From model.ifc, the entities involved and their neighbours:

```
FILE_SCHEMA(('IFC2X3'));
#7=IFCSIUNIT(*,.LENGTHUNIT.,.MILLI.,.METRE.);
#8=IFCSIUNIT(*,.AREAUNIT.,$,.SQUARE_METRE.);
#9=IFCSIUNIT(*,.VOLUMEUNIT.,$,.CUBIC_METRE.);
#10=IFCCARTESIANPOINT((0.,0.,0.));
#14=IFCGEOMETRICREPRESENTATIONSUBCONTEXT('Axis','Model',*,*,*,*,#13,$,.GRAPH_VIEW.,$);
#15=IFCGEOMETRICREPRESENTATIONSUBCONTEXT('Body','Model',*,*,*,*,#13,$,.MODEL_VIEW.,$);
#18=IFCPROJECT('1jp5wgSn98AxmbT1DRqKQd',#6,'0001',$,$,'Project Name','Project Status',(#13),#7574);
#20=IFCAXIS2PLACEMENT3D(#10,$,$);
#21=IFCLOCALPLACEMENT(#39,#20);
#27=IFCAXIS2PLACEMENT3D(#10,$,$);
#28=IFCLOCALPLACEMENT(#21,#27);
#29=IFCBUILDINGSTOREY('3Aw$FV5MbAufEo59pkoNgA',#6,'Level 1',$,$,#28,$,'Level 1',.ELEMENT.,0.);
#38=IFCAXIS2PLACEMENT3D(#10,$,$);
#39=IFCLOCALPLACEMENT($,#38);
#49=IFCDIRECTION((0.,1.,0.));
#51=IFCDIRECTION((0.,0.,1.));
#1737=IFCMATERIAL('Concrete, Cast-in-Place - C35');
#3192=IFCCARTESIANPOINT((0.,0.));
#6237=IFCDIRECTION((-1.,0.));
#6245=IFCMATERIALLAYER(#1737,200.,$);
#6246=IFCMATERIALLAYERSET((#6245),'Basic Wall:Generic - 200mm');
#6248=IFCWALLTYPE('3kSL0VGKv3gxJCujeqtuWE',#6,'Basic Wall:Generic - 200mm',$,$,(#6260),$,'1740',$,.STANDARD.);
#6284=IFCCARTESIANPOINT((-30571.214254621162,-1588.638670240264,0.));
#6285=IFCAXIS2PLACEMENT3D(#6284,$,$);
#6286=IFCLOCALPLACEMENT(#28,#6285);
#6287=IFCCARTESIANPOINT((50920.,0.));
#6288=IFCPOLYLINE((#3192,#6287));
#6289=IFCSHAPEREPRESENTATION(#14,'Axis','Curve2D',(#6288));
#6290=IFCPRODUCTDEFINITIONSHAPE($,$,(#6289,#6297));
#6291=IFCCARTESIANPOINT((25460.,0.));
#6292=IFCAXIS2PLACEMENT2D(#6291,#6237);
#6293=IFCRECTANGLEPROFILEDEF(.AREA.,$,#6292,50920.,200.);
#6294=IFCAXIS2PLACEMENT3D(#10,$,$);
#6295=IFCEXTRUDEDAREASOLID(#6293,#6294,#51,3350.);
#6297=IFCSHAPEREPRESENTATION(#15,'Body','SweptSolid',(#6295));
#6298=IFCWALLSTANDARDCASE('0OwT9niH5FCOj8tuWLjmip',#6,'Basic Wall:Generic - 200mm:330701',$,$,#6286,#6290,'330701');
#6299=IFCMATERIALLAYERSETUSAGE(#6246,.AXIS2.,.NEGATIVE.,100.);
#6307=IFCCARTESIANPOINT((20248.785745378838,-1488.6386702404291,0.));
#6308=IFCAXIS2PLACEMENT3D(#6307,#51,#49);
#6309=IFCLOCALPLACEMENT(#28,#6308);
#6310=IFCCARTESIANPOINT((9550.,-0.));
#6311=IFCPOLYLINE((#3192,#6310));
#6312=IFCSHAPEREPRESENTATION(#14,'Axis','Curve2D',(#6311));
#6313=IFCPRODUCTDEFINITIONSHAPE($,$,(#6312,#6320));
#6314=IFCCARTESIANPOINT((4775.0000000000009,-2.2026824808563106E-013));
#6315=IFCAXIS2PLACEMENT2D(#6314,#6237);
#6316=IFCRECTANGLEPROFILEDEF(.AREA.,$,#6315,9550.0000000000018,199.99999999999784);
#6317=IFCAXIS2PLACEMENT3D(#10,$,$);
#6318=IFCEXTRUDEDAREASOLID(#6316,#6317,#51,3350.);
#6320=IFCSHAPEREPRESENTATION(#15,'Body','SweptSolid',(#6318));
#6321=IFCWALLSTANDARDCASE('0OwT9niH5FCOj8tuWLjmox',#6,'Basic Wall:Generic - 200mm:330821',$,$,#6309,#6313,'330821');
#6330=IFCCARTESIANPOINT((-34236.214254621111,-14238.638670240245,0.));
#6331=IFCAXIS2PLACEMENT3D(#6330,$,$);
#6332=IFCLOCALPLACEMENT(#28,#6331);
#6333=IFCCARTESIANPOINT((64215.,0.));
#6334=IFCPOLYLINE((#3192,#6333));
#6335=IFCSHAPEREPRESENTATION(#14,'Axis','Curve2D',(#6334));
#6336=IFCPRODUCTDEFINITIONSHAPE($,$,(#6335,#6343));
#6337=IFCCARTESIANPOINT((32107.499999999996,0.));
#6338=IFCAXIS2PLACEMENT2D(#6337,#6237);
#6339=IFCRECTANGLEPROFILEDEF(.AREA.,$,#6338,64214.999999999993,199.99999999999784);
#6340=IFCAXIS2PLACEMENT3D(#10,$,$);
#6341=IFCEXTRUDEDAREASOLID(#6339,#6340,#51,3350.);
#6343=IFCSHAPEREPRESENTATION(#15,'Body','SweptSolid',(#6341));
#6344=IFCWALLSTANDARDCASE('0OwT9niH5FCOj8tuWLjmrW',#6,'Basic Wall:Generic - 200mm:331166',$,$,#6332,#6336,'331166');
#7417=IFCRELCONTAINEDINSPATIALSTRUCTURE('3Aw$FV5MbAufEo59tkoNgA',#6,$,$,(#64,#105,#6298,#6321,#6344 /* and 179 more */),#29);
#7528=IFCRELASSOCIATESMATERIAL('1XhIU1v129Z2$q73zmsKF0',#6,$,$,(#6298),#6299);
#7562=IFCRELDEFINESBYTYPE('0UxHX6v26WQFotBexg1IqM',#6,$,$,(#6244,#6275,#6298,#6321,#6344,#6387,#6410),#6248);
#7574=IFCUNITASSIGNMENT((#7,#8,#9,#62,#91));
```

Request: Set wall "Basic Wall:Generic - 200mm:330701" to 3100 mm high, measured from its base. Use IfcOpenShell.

```python
import ifcopenshell
import ifcopenshell.geom
import ifcopenshell.util.representation
import ifcopenshell.util.shape
import ifcopenshell.util.unit

model = ifcopenshell.open("model.ifc")
unit_scale = ifcopenshell.util.unit.calculate_unit_scale(model)
settings = ifcopenshell.geom.settings()


def volume(element):
    """Net volume in cubic metres, openings subtracted."""
    shape = ifcopenshell.geom.create_shape(settings, element)
    return ifcopenshell.util.shape.get_volume(shape.geometry)


wall = model.by_guid("0OwT9niH5FCOj8tuWLjmip")
before = volume(wall)

body = ifcopenshell.util.representation.get_representation(wall, "Model", "Body")
solid = body.Items[0]
old_height = solid.Depth
solid.Depth = 3.1 / unit_scale
after = volume(wall)

print(f"height {old_height:g} -> {solid.Depth:g}, volume {before:.3f} -> {after:.3f} m3")

model.write("model_v2.ifc")
```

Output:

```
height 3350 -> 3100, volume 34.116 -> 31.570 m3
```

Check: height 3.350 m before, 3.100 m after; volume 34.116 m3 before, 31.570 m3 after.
